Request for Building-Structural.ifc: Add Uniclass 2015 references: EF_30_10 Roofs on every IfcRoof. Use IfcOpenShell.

First a look at what the model holds.

```python
import ifcopenshell

model = ifcopenshell.open("Building-Structural.ifc")
print(model.schema)
print("classifications:", [c.Name for c in model.by_type("IfcClassification")])
for ifc_class in ("IfcDoor", "IfcRoof", "IfcStair", "IfcWall", "IfcWindow"):
    print(ifc_class, len(model.by_type(ifc_class)))
```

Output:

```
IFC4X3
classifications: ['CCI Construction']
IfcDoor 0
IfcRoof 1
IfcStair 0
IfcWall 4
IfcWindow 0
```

```python
import ifcopenshell
import ifcopenshell.api.classification

model = ifcopenshell.open("Building-Structural.ifc")

system = ifcopenshell.api.classification.add_classification(model, classification="Uniclass 2015")

codes = {
    "IfcRoof": ("EF_30_10", "Roofs"),
}
for ifc_class, (code, name) in codes.items():
    products = model.by_type(ifc_class)
    ifcopenshell.api.classification.add_reference(
        model, products=products, classification=system, identification=code, name=name
    )
    print(code, len(products))

model.write("Building-Structural_rev.ifc")
```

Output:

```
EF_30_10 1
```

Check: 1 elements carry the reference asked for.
